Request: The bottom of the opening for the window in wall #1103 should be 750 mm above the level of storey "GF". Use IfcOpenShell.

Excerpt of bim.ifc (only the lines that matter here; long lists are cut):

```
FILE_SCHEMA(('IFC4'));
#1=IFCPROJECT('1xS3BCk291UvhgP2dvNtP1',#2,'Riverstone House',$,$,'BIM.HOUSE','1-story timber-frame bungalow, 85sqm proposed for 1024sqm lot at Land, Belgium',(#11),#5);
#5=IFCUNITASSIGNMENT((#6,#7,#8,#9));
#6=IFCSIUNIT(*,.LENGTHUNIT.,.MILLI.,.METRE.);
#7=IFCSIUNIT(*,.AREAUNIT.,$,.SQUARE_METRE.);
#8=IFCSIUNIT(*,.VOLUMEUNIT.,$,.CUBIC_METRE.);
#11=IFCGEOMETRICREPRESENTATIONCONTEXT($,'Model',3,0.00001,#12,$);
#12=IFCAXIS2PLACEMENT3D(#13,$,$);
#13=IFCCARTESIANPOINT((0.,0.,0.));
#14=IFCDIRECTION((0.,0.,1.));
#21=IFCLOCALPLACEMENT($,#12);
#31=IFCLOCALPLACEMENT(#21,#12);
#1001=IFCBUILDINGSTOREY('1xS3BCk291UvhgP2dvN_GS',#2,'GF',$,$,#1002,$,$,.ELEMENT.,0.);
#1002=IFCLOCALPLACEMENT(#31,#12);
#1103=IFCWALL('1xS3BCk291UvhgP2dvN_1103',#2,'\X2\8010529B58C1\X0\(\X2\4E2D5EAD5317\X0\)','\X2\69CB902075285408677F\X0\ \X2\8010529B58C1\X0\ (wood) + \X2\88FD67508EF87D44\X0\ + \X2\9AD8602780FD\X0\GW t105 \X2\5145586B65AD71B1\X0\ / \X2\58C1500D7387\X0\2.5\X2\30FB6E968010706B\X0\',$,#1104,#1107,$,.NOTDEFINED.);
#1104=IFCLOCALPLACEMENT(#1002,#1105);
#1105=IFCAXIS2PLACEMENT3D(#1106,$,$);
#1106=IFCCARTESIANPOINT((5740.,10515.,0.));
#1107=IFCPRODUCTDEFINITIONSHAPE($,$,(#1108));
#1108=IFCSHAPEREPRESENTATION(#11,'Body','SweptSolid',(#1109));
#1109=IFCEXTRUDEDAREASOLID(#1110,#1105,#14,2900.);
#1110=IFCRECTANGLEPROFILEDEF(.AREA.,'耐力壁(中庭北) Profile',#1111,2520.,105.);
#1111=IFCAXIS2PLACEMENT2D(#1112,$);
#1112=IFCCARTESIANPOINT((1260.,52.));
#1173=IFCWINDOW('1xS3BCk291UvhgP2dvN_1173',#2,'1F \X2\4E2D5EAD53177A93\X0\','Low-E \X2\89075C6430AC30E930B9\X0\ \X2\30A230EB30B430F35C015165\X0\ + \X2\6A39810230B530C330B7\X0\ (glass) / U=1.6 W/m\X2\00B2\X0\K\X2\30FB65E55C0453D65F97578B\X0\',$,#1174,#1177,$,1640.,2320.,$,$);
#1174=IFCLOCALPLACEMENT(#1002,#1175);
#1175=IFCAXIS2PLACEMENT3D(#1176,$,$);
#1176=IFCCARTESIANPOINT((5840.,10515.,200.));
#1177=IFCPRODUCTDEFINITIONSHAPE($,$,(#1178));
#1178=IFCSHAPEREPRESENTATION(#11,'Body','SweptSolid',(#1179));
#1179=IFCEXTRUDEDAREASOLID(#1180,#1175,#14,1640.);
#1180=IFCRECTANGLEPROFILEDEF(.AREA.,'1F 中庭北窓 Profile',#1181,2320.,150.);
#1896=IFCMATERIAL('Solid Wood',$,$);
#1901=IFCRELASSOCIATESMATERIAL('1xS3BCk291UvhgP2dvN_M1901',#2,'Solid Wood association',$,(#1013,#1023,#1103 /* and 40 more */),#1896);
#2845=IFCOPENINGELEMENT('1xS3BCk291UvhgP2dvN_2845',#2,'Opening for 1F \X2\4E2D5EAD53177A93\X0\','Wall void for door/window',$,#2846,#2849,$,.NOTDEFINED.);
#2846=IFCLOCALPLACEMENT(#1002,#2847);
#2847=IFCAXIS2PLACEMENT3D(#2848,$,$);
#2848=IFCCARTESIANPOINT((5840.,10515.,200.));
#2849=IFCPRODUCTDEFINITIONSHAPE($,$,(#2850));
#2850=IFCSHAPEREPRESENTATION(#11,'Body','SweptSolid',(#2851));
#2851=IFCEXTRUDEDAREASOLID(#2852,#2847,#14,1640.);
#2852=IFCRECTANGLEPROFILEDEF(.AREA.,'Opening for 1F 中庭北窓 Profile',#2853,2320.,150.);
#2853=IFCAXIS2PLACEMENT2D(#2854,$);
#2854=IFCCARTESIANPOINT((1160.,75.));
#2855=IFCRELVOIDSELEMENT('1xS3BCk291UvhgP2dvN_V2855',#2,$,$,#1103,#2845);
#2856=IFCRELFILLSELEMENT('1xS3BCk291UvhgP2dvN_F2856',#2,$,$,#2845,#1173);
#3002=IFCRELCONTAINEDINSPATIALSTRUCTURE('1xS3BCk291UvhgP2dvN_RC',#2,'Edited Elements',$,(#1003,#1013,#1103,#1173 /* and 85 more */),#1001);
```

```python
import numpy as np
import ifcopenshell
import ifcopenshell.api.geometry
import ifcopenshell.geom
import ifcopenshell.util.element
import ifcopenshell.util.placement
import ifcopenshell.util.shape
import ifcopenshell.util.unit

model = ifcopenshell.open("bim.ifc")
unit_scale = ifcopenshell.util.unit.calculate_unit_scale(model)

window = model.by_id(1173)
opening = window.FillsVoids[0].RelatingOpeningElement
storey = ifcopenshell.util.element.get_container(window, ifc_class="IfcBuildingStorey")
level = ifcopenshell.util.placement.get_local_placement(storey.ObjectPlacement)[2, 3]

# The opening's origin need not be at the sill, so measure its lowest point.
shape = ifcopenshell.geom.create_shape(ifcopenshell.geom.settings(), opening)
bottom = ifcopenshell.util.shape.get_shape_bottom_elevation(shape, shape.geometry) / unit_scale
dz = level + 0.75 / unit_scale - bottom

shift = np.array([0.0, 0.0, dz])
# The window is not placed relative to its opening, so move both.
for product in (opening, window):
    matrix = ifcopenshell.util.placement.get_local_placement(product.ObjectPlacement)
    matrix[:3, 3] += shift
    ifcopenshell.api.geometry.edit_object_placement(model, product=product, matrix=matrix, is_si=False)

print(f"moved by {dz * unit_scale:+.3f} m")

model.write("bim-out.ifc")
```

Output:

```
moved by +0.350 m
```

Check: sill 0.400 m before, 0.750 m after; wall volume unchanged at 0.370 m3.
